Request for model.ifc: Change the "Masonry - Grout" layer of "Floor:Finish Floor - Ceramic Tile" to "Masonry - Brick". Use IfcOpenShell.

First a look at what the model holds.

```python
import ifcopenshell
import ifcopenshell.util.element

model = ifcopenshell.open("model.ifc")
print(model.schema)
for layer_set in model.by_type("IfcMaterialLayerSet"):
    if layer_set.LayerSetName == "Floor:Finish Floor - Ceramic Tile":
        for layer in layer_set.MaterialLayers:
            print(layer.id(), layer.Material and layer.Material.Name, layer.LayerThickness, sep=" | ")
        print(len(ifcopenshell.util.element.get_elements_by_material(model, layer_set)), "elements and types use it")
print(sorted(m.Name for m in model.by_type("IfcMaterial") if m.Name)[:60])
```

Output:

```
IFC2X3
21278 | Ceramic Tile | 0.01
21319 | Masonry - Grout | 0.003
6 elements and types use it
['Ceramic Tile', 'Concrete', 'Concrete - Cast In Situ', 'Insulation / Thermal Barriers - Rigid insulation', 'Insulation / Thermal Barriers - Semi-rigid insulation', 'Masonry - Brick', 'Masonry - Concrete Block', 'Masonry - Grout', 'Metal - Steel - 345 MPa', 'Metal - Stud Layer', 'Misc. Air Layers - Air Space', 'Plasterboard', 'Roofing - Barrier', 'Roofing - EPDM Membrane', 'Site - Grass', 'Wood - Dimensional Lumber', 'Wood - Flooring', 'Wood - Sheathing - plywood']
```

```python
import ifcopenshell
import ifcopenshell.api.material

model = ifcopenshell.open("model.ifc")

layer_set = next(s for s in model.by_type("IfcMaterialLayerSet") if s.LayerSetName == "Floor:Finish Floor - Ceramic Tile")
layer = next(l for l in layer_set.MaterialLayers if l.Material and l.Material.Name == "Masonry - Grout")
material = next(m for m in model.by_type("IfcMaterial") if m.Name == "Masonry - Brick")

# Point this one layer at the other material; renaming the old one would change it everywhere.
ifcopenshell.api.material.edit_layer(model, layer=layer, attributes={}, material=material)

print([l.Material.Name if l.Material else None for l in layer_set.MaterialLayers])

model.write("model_rev.ifc")
```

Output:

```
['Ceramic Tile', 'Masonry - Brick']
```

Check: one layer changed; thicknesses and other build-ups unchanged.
